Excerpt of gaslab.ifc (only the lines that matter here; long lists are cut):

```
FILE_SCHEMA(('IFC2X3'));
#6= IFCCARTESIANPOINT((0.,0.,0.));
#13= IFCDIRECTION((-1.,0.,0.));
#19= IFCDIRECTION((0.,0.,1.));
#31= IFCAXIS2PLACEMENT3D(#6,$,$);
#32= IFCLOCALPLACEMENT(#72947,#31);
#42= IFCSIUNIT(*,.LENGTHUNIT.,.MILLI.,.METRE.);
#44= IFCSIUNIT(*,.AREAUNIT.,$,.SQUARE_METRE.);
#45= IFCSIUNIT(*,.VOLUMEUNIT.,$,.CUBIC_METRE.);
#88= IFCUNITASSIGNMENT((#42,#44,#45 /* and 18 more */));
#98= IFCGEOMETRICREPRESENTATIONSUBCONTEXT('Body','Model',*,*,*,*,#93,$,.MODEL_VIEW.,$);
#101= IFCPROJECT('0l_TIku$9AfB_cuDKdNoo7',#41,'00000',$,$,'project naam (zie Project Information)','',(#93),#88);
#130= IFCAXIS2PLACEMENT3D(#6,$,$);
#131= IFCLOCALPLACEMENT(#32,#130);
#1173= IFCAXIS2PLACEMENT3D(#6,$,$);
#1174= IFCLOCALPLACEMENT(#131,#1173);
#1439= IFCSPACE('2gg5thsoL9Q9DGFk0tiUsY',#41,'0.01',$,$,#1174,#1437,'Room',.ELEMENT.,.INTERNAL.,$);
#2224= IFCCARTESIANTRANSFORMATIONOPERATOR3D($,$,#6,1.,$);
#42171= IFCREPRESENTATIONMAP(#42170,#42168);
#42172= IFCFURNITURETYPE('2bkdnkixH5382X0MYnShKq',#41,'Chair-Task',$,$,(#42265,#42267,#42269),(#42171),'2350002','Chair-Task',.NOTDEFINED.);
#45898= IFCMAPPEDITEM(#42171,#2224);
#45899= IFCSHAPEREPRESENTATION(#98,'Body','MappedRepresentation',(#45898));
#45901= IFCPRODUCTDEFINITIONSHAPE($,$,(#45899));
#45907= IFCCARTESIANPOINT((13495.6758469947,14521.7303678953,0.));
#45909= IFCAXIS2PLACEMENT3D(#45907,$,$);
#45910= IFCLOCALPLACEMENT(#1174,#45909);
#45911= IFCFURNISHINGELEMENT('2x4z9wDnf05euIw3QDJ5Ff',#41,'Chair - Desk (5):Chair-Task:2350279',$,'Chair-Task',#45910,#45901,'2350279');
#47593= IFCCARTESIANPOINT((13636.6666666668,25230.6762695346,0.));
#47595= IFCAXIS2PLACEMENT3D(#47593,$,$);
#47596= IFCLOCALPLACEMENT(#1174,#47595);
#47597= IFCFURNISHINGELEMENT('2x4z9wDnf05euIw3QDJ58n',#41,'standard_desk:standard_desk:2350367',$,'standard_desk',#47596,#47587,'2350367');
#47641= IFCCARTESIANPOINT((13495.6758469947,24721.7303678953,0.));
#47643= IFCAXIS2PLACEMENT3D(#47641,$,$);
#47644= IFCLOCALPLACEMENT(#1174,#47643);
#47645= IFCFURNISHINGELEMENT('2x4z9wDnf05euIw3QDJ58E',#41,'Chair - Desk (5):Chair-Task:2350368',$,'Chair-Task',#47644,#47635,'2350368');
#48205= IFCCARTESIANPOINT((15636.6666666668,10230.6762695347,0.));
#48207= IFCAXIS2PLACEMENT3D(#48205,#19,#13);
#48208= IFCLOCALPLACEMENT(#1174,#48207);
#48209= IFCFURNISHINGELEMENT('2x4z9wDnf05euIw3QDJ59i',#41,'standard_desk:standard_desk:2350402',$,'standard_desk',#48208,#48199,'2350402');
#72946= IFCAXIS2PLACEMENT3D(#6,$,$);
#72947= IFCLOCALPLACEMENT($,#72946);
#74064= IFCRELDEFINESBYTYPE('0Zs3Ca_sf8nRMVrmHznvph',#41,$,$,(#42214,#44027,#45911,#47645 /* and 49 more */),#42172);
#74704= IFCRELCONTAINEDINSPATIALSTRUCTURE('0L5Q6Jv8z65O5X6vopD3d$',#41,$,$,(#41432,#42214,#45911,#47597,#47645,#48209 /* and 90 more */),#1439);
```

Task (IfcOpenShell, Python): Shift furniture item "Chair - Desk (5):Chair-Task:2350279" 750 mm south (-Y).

```python
import ifcopenshell
import ifcopenshell.api.geometry
import ifcopenshell.util.placement
import ifcopenshell.util.unit

model = ifcopenshell.open("gaslab.ifc")
unit_scale = ifcopenshell.util.unit.calculate_unit_scale(model)

item = model.by_guid("2x4z9wDnf05euIw3QDJ5Ff")
matrix = ifcopenshell.util.placement.get_local_placement(item.ObjectPlacement)
matrix[1, 3] -= 0.75 / unit_scale
ifcopenshell.api.geometry.edit_object_placement(model, product=item, matrix=matrix, is_si=False)

print(ifcopenshell.util.placement.get_local_placement(item.ObjectPlacement).round(3) + 0.0)

model.write("gaslab-out.ifc")
```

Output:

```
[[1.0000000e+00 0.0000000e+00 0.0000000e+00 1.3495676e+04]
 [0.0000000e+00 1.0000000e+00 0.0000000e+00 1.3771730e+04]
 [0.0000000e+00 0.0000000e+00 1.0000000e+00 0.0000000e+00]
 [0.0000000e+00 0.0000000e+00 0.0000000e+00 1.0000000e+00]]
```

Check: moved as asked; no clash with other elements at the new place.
